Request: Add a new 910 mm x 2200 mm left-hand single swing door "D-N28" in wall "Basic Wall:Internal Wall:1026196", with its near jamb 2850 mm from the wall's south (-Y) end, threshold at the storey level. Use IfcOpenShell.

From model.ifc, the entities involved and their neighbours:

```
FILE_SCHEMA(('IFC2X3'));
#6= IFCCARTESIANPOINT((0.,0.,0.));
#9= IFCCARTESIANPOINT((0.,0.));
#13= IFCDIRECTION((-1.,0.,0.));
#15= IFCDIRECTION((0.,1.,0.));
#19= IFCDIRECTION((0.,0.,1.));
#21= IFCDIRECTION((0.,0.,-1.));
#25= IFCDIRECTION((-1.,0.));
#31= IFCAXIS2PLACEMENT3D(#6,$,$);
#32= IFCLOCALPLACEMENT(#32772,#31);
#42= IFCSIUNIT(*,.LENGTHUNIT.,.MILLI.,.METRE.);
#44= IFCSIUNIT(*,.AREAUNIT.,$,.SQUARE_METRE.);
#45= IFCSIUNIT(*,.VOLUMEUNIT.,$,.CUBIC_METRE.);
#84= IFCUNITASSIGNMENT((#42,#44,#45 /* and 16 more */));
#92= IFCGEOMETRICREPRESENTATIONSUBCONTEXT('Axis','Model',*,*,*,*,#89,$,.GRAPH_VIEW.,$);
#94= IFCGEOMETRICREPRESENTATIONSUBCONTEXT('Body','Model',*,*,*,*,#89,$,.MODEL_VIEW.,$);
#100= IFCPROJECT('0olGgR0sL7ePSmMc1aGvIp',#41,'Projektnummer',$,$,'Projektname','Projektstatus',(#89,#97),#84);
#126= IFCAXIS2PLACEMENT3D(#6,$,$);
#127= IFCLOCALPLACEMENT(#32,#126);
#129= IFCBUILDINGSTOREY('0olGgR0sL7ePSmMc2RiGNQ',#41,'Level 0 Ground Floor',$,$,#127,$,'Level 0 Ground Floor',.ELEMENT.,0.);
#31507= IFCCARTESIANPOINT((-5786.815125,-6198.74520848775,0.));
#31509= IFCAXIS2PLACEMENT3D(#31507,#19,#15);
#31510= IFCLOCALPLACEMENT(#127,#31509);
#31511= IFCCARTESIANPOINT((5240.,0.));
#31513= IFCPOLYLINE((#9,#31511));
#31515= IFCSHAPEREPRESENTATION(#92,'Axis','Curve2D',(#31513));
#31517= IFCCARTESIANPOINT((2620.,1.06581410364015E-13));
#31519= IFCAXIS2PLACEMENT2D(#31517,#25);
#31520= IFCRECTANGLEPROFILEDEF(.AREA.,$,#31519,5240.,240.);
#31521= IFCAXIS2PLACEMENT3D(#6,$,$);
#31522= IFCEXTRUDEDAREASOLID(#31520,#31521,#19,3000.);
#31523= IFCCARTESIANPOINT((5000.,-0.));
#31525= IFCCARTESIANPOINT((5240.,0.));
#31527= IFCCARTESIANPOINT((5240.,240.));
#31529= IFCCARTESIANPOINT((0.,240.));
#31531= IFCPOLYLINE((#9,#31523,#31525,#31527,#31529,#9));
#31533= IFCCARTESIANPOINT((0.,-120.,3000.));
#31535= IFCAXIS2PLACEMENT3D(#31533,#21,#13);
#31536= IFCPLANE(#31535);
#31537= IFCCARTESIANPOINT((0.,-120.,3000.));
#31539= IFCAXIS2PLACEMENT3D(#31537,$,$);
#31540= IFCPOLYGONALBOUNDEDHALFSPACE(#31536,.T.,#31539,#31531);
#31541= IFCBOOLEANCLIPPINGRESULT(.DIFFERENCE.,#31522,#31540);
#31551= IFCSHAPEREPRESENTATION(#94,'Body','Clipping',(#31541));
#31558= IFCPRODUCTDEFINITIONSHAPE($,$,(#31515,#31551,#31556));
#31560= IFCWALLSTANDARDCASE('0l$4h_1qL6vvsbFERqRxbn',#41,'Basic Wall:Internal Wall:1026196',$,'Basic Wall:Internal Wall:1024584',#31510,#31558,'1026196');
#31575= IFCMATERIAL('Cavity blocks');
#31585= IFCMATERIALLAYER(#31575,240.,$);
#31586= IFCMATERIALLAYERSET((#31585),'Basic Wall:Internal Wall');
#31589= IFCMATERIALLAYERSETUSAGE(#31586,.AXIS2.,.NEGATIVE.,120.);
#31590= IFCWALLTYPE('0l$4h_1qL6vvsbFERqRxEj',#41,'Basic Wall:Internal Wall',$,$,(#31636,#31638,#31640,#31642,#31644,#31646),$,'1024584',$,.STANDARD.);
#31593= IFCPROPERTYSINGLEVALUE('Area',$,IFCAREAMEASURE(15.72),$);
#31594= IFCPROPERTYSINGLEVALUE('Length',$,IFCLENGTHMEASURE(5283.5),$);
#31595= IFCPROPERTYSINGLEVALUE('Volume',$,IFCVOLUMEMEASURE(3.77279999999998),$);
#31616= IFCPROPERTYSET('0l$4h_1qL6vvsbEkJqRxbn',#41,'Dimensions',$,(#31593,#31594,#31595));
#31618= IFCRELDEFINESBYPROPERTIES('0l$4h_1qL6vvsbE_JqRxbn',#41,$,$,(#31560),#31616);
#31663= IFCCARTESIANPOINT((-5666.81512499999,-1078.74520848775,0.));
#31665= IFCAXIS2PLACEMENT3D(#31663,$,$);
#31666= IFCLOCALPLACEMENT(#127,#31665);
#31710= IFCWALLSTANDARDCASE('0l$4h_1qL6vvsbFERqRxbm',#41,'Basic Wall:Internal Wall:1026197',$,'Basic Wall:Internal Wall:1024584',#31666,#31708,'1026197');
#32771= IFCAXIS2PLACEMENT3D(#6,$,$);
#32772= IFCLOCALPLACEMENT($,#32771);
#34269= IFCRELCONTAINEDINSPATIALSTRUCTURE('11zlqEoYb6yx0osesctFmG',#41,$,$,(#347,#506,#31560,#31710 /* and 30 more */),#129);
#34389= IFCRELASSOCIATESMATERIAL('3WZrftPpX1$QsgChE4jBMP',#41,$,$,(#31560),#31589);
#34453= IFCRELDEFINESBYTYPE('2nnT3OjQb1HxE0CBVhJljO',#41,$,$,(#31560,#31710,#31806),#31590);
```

```python
import numpy as np
import ifcopenshell
import ifcopenshell.api.feature
import ifcopenshell.api.geometry
import ifcopenshell.api.pset
import ifcopenshell.api.root
import ifcopenshell.api.spatial
import ifcopenshell.api.type
import ifcopenshell.geom
import ifcopenshell.util.element
import ifcopenshell.util.placement
import ifcopenshell.util.representation
import ifcopenshell.util.shape
import ifcopenshell.util.unit

model = ifcopenshell.open("model.ifc")
unit_scale = ifcopenshell.util.unit.calculate_unit_scale(model)
area_scale = ifcopenshell.util.unit.calculate_unit_scale(model, "AREAUNIT")
volume_scale = ifcopenshell.util.unit.calculate_unit_scale(model, "VOLUMEUNIT")
settings = ifcopenshell.geom.settings()


def volume(element):
    """Net volume in cubic metres, openings subtracted."""
    shape = ifcopenshell.geom.create_shape(settings, element)
    return ifcopenshell.util.shape.get_volume(shape.geometry)


wall = model.by_id(31560)
storey = ifcopenshell.util.element.get_container(wall, ifc_class="IfcBuildingStorey")
context = ifcopenshell.util.representation.get_context(model, "Model", "Body", "MODEL_VIEW")
before = volume(wall)

width, height, from_end, sill = 0.91, 2.2, 2.85, 0.0  # metres

# The wall runs along its own X axis, and the end named is its -X end.
wall_shape = ifcopenshell.geom.create_shape(settings, wall)
x, y, z = ifcopenshell.util.shape.get_vertices(wall_shape.geometry).T
start = x.min() + from_end
face, thickness = float(y.min()), float(y.max() - y.min())
wall_matrix = ifcopenshell.util.placement.get_local_placement(wall.ObjectPlacement)
level = ifcopenshell.util.placement.get_local_placement(storey.ObjectPlacement)[2, 3]


def in_wall(x, y):
    """Placement at x, y metres in the wall's axes, at sill height."""
    matrix = wall_matrix.copy()
    matrix[:, 3] = wall_matrix @ np.array([x / unit_scale, y / unit_scale, 0.0, 1.0])
    matrix[2, 3] = level + sill / unit_scale
    return matrix


# Opening: a box that overshoots both wall faces by 50 mm.
opening = ifcopenshell.api.root.create_entity(model, ifc_class="IfcOpeningElement")
box = ifcopenshell.api.geometry.add_wall_representation(
    model, context=context, length=width, height=height, thickness=thickness + 0.1
)
ifcopenshell.api.geometry.assign_representation(model, product=opening, representation=box)
ifcopenshell.api.geometry.edit_object_placement(model, product=opening, matrix=in_wall(start, face - 0.05), is_si=False)
ifcopenshell.api.feature.add_feature(model, feature=opening, element=wall)

door = ifcopenshell.api.root.create_entity(model, ifc_class="IfcDoor", name="D-N28")
door.OverallWidth, door.OverallHeight = width / unit_scale, height / unit_scale
body = ifcopenshell.api.geometry.add_door_representation(
    model,
    context=context,
    overall_width=door.OverallWidth,
    overall_height=door.OverallHeight,
    operation_type="SINGLE_SWING_LEFT",
    lining_properties={"LiningDepth": thickness / unit_scale, "ThresholdDepth": thickness / unit_scale},
)
ifcopenshell.api.geometry.assign_representation(model, product=door, representation=body)
ifcopenshell.api.spatial.assign_container(model, products=[door], relating_structure=storey)
fills = ifcopenshell.api.feature.add_filling(model, opening=opening, element=door)
fills.OwnerHistory = door.OwnerHistory  # required in IFC2X3

# IFC2X3 keeps the operation on the door style.
style = ifcopenshell.api.root.create_entity(model, ifc_class="IfcDoorStyle", name="D-N28")
style.OperationType, style.ConstructionType = "SINGLE_SWING_LEFT", "NOTDEFINED"
style.ParameterTakesPrecedence = style.Sizeable = False
ifcopenshell.api.type.assign_type(model, related_objects=[door], relating_type=style)

# The lining spans the wall, so the door starts at the wall face.
ifcopenshell.api.geometry.edit_object_placement(model, product=door, matrix=in_wall(start, face), is_si=False)

after = volume(wall)

# Update the wall's stored quantities.
pset = model.by_id(ifcopenshell.util.element.get_pset(wall, "Dimensions", should_inherit=False)["id"])
ifcopenshell.api.pset.edit_pset(model, pset=pset, properties={
    "Area": model.create_entity("IfcAreaMeasure", after / thickness / area_scale),
    "Volume": model.create_entity("IfcVolumeMeasure", after / volume_scale),
})

print(f"wall volume {before:.3f} -> {after:.3f} m3")

model.write("model_updated.ifc")
```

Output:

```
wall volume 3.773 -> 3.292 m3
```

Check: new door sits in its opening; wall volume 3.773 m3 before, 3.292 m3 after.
